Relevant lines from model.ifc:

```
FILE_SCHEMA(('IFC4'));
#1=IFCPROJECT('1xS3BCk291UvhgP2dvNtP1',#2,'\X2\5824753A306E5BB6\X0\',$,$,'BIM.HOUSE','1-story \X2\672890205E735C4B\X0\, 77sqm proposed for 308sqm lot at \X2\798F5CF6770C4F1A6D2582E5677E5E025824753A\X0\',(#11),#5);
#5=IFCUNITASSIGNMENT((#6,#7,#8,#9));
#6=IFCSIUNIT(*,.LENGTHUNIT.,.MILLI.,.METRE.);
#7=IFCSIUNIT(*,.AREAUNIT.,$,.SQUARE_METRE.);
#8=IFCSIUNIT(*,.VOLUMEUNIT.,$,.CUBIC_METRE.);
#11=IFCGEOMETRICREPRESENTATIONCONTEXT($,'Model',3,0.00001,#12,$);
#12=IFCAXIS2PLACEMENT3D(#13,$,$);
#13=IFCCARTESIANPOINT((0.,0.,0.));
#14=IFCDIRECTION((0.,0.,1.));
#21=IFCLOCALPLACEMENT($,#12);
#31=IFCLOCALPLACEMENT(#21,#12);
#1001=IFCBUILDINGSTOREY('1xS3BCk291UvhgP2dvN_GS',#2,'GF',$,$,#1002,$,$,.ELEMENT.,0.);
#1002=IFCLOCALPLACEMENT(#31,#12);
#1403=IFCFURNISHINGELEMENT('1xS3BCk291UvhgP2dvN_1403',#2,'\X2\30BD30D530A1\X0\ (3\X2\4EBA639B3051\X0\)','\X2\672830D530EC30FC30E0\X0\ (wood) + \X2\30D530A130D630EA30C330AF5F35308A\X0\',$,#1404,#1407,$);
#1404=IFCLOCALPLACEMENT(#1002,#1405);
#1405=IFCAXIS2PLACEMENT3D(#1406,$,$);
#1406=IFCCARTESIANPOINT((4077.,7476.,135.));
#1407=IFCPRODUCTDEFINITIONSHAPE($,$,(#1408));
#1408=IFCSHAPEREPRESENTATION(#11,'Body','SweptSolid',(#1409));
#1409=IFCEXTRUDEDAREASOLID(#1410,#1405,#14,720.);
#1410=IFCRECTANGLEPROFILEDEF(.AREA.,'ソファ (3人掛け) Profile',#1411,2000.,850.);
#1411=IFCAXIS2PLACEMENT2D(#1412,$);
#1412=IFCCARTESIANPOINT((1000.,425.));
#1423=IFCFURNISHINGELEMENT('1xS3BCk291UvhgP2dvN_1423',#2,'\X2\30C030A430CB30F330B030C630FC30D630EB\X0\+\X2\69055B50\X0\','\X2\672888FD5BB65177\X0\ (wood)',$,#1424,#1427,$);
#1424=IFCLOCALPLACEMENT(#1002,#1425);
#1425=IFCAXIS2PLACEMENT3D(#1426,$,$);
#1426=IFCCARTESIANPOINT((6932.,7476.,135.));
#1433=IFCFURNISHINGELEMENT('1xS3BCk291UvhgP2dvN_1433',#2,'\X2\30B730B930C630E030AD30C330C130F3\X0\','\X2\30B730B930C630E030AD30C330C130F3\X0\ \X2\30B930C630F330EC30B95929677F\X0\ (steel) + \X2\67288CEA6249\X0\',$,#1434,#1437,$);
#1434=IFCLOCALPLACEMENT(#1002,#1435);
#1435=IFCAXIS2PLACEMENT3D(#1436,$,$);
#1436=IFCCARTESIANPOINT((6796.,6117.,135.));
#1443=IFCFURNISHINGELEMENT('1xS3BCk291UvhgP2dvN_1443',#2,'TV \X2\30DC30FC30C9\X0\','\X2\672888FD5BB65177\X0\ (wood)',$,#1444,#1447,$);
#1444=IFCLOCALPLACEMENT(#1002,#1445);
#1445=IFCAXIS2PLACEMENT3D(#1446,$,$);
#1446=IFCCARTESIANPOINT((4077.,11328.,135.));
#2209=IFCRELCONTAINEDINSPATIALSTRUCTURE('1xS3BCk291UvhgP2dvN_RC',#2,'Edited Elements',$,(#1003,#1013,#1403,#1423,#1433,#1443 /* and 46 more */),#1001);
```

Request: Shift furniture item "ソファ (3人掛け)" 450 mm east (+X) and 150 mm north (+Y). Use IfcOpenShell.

```python
import ifcopenshell
import ifcopenshell.api.geometry
import ifcopenshell.util.placement
import ifcopenshell.util.unit

model = ifcopenshell.open("model.ifc")
unit_scale = ifcopenshell.util.unit.calculate_unit_scale(model)

item = model.by_guid("1xS3BCk291UvhgP2dvN_1403")
matrix = ifcopenshell.util.placement.get_local_placement(item.ObjectPlacement)
matrix[0, 3] += 0.45 / unit_scale
matrix[1, 3] += 0.15 / unit_scale
ifcopenshell.api.geometry.edit_object_placement(model, product=item, matrix=matrix, is_si=False)

print(ifcopenshell.util.placement.get_local_placement(item.ObjectPlacement).round(3) + 0.0)

model.write("model_rev.ifc")
```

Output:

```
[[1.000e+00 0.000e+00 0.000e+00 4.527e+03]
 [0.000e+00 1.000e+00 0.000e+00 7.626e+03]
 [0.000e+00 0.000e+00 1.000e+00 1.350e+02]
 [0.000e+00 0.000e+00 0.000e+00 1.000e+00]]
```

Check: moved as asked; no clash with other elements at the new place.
